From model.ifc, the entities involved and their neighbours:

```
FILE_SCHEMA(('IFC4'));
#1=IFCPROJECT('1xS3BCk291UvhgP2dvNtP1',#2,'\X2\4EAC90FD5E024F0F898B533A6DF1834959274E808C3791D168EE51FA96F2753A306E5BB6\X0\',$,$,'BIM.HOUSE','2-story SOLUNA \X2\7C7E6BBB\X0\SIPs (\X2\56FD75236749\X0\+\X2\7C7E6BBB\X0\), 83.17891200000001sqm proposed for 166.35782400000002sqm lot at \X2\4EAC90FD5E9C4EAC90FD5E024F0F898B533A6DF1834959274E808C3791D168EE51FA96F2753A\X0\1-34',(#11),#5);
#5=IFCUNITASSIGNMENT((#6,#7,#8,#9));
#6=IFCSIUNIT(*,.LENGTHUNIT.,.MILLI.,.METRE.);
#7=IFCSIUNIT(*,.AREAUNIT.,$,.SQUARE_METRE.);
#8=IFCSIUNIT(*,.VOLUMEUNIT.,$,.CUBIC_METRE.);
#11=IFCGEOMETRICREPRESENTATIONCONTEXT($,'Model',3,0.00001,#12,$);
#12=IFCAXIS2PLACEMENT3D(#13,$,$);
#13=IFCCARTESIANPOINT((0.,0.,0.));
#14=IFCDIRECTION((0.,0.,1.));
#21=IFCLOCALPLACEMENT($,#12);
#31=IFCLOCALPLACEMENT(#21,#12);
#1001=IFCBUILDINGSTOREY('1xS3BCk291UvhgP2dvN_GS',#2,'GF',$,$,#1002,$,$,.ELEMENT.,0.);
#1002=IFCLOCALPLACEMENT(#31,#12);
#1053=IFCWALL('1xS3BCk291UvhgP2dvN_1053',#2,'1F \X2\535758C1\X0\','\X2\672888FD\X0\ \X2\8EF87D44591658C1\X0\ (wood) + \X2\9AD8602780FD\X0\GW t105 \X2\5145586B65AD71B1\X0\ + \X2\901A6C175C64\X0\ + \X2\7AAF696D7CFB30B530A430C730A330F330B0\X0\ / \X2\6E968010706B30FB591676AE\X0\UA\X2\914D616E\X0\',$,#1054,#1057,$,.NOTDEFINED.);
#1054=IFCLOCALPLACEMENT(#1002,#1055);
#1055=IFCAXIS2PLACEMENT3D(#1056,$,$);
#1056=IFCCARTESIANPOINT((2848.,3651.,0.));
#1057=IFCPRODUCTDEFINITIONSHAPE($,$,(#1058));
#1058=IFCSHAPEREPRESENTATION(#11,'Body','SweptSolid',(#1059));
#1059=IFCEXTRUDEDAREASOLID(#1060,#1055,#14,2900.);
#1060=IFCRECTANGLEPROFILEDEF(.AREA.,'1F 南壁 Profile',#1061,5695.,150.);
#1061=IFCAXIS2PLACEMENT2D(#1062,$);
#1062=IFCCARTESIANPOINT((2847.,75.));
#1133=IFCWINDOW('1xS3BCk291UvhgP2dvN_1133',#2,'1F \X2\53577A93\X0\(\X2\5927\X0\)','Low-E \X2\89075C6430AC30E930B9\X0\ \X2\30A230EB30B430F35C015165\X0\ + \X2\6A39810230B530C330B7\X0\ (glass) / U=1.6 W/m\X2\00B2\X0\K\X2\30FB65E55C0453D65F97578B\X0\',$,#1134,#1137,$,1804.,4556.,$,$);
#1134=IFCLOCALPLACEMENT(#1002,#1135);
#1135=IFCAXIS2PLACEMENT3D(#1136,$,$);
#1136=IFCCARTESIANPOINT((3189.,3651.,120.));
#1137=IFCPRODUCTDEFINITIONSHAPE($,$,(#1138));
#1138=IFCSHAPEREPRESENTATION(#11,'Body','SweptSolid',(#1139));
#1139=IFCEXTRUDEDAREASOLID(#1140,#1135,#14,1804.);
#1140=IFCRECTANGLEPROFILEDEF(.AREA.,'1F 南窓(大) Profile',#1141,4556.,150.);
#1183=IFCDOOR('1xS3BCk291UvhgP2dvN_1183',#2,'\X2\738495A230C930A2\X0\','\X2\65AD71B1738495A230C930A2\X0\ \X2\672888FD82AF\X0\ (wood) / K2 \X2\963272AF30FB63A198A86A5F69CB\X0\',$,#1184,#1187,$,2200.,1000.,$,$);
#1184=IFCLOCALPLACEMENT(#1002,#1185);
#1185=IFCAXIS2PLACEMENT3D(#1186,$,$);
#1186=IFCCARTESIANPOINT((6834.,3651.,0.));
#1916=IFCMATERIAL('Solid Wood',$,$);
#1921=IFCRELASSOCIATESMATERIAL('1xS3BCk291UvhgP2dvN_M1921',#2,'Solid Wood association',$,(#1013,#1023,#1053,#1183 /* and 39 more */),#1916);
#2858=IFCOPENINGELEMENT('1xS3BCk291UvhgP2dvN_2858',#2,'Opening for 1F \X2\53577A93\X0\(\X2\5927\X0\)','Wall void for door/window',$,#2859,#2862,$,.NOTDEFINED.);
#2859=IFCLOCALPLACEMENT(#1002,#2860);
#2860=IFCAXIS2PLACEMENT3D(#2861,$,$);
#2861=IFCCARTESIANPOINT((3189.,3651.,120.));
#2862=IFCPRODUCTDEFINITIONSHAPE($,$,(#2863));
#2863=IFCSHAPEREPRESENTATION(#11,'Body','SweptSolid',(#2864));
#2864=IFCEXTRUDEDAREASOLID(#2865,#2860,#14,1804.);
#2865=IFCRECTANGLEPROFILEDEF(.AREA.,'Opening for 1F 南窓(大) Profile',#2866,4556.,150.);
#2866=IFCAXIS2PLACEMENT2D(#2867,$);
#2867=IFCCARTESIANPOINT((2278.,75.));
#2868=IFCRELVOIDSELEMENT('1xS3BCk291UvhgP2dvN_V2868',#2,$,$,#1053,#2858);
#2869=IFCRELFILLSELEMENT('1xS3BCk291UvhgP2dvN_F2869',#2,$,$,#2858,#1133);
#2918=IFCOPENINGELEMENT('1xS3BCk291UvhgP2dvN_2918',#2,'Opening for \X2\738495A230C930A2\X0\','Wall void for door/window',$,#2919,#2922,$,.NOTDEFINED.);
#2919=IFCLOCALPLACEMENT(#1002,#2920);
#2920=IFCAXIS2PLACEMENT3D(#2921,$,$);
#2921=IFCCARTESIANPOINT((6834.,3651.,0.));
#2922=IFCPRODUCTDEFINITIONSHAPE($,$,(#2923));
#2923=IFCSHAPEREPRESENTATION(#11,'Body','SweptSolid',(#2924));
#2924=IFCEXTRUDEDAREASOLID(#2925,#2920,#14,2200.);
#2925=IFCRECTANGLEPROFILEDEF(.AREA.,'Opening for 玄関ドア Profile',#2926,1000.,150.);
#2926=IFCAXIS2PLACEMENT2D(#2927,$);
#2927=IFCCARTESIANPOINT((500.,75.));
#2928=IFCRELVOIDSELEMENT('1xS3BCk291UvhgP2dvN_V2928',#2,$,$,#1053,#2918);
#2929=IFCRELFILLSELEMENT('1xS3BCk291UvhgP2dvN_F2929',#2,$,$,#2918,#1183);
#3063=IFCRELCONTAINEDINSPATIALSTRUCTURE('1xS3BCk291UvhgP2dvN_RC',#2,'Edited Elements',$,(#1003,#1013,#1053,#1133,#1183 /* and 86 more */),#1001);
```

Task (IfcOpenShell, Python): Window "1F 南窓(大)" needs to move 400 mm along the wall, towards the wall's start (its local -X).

```python
import ifcopenshell
import ifcopenshell.api.geometry
import ifcopenshell.util.placement
import ifcopenshell.util.unit

model = ifcopenshell.open("model.ifc")
unit_scale = ifcopenshell.util.unit.calculate_unit_scale(model)

window = model.by_id(1133)
opening = window.FillsVoids[0].RelatingOpeningElement
wall = opening.VoidsElements[0].RelatingBuildingElement

wall_matrix = ifcopenshell.util.placement.get_local_placement(wall.ObjectPlacement)
shift = wall_matrix[:3, 0] * -0.4 / unit_scale
before = ifcopenshell.util.placement.get_local_placement(window.ObjectPlacement)[:3, 3].copy()

# The window is not placed relative to its opening, so move both.
for product in (opening, window):
    matrix = ifcopenshell.util.placement.get_local_placement(product.ObjectPlacement)
    matrix[:3, 3] += shift
    ifcopenshell.api.geometry.edit_object_placement(model, product=product, matrix=matrix, is_si=False)

after = ifcopenshell.util.placement.get_local_placement(window.ObjectPlacement)[:3, 3]
print("window moved by", (after - before).round(3) + 0.0)

model.write("model_v2.ifc")
```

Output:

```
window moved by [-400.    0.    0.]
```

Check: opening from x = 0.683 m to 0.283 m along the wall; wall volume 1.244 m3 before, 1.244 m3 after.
